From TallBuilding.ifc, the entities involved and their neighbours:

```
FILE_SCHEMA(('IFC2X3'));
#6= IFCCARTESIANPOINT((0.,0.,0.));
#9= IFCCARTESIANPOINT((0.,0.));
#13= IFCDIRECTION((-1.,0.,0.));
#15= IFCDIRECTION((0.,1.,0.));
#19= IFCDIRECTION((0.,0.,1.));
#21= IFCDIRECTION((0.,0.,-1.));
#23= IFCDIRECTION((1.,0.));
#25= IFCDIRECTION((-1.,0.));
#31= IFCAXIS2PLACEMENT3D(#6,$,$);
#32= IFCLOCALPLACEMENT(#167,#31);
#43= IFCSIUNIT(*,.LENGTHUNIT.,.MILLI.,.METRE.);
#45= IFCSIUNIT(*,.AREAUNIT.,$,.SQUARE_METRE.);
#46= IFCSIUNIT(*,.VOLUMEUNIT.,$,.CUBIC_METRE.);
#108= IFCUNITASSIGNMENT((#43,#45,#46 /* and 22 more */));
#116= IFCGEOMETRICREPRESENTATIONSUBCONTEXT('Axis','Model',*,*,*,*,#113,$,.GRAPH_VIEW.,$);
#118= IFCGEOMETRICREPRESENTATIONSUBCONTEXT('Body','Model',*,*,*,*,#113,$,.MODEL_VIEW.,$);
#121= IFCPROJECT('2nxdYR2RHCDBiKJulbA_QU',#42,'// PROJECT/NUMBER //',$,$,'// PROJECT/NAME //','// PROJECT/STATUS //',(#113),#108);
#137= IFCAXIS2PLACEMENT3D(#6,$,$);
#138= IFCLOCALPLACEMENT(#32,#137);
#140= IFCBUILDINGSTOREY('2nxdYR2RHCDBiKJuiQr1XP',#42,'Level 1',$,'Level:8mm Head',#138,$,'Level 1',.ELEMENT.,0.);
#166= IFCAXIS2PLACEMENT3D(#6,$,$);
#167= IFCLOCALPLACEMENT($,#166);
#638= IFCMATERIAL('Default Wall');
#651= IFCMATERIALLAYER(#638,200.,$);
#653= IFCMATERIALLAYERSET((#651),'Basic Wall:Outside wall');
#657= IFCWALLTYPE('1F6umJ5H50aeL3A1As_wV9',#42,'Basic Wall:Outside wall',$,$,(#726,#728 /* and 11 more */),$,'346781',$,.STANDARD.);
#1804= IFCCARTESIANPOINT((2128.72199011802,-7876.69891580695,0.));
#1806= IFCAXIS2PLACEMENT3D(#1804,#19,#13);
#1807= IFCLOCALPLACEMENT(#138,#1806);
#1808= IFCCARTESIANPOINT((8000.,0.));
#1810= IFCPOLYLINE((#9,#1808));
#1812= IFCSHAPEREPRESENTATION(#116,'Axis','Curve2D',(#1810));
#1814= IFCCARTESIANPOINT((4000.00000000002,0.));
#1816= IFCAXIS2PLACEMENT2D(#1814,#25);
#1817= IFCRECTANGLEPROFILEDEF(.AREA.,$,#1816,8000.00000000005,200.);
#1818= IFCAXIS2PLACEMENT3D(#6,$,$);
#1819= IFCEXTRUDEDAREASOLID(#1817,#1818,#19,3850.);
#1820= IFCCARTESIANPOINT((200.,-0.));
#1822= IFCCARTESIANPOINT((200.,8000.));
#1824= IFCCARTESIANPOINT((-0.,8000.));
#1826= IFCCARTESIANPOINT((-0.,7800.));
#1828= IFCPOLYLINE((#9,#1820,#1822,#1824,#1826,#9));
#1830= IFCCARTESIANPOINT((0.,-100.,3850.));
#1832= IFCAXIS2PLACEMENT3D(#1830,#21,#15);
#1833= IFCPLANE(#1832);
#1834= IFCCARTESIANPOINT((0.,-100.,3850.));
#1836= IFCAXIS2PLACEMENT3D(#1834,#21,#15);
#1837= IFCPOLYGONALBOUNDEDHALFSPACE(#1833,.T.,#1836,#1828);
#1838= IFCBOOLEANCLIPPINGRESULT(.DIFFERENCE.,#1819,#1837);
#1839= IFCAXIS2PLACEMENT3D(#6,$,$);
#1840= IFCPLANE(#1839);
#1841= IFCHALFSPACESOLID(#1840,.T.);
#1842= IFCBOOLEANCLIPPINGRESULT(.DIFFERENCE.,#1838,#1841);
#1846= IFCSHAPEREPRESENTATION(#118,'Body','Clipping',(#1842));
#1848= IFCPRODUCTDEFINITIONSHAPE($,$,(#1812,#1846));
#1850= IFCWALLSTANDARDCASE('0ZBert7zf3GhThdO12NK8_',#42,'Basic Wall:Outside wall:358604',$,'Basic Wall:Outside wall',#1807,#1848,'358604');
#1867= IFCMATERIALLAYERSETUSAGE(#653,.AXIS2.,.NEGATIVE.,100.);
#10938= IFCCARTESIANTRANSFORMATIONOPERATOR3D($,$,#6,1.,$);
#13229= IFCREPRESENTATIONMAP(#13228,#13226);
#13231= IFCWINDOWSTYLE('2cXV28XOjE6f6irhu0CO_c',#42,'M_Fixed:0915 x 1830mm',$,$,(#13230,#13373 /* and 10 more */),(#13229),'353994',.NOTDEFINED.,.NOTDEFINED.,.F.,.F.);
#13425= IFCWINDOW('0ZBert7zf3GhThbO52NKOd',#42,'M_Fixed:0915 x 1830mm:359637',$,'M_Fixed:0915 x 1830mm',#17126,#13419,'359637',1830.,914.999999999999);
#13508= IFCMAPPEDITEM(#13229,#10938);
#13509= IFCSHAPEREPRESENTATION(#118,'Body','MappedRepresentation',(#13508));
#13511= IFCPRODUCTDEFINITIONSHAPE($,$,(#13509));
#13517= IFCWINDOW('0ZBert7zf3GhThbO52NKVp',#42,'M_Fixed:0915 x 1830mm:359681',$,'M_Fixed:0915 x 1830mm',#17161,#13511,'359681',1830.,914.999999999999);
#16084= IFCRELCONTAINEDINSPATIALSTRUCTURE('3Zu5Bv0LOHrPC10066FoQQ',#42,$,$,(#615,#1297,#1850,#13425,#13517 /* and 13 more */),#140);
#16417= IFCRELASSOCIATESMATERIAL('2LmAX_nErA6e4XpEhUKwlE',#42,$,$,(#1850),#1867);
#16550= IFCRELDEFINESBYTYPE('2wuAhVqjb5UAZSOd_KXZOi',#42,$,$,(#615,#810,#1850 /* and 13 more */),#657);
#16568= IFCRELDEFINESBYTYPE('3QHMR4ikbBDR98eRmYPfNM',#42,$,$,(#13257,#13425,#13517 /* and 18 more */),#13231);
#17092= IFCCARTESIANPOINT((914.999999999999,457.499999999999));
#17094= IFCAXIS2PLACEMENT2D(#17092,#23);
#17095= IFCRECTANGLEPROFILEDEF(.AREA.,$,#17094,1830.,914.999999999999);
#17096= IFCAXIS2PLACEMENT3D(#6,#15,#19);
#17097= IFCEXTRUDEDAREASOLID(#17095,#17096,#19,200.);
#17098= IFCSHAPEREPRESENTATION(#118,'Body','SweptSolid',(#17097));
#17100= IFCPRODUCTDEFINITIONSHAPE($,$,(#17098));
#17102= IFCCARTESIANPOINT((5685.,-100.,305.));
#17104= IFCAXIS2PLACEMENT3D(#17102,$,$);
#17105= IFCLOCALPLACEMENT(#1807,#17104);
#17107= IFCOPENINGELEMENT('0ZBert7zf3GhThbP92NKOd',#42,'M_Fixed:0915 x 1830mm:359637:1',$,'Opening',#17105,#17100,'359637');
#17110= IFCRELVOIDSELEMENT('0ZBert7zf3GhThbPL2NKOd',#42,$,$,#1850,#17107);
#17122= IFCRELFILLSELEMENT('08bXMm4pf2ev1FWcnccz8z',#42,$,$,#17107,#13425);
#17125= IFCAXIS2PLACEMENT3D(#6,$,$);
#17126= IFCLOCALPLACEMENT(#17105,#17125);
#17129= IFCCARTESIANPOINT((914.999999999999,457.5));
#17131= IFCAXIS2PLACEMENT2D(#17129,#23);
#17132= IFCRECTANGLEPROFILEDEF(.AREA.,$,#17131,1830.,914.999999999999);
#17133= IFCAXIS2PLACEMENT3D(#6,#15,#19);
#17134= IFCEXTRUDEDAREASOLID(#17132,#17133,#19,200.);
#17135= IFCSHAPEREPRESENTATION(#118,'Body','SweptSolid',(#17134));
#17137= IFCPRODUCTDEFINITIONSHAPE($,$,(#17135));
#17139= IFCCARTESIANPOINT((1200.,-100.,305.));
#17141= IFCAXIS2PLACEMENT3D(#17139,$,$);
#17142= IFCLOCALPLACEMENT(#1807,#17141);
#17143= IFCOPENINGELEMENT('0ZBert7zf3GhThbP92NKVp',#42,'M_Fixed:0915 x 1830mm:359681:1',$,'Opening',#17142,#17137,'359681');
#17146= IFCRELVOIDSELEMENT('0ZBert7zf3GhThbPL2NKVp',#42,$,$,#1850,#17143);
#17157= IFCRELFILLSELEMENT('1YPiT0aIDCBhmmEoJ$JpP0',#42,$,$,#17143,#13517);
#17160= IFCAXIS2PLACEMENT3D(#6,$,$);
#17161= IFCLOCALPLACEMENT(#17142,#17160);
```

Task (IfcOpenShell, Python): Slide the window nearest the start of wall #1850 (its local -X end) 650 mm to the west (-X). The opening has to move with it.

```python
import ifcopenshell
import ifcopenshell.api.geometry
import ifcopenshell.util.placement
import ifcopenshell.util.unit

model = ifcopenshell.open("TallBuilding.ifc")
unit_scale = ifcopenshell.util.unit.calculate_unit_scale(model)

window = model.by_id(13517)
opening = window.FillsVoids[0].RelatingOpeningElement
wall = opening.VoidsElements[0].RelatingBuildingElement

wall_matrix = ifcopenshell.util.placement.get_local_placement(wall.ObjectPlacement)
shift = wall_matrix[:3, 0] * 0.65 / unit_scale
before = ifcopenshell.util.placement.get_local_placement(window.ObjectPlacement)[:3, 3].copy()

# The window is placed relative to its opening, so it follows when the opening moves.
matrix = ifcopenshell.util.placement.get_local_placement(opening.ObjectPlacement)
matrix[:3, 3] += shift
ifcopenshell.api.geometry.edit_object_placement(
    model, product=opening, matrix=matrix, is_si=False, should_transform_children=True
)

after = ifcopenshell.util.placement.get_local_placement(window.ObjectPlacement)[:3, 3]
print("window moved by", (after - before).round(3) + 0.0)

model.write("TallBuilding_v2.ifc")
```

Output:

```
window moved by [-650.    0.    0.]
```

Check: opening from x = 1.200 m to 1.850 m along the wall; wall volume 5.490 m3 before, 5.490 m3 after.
